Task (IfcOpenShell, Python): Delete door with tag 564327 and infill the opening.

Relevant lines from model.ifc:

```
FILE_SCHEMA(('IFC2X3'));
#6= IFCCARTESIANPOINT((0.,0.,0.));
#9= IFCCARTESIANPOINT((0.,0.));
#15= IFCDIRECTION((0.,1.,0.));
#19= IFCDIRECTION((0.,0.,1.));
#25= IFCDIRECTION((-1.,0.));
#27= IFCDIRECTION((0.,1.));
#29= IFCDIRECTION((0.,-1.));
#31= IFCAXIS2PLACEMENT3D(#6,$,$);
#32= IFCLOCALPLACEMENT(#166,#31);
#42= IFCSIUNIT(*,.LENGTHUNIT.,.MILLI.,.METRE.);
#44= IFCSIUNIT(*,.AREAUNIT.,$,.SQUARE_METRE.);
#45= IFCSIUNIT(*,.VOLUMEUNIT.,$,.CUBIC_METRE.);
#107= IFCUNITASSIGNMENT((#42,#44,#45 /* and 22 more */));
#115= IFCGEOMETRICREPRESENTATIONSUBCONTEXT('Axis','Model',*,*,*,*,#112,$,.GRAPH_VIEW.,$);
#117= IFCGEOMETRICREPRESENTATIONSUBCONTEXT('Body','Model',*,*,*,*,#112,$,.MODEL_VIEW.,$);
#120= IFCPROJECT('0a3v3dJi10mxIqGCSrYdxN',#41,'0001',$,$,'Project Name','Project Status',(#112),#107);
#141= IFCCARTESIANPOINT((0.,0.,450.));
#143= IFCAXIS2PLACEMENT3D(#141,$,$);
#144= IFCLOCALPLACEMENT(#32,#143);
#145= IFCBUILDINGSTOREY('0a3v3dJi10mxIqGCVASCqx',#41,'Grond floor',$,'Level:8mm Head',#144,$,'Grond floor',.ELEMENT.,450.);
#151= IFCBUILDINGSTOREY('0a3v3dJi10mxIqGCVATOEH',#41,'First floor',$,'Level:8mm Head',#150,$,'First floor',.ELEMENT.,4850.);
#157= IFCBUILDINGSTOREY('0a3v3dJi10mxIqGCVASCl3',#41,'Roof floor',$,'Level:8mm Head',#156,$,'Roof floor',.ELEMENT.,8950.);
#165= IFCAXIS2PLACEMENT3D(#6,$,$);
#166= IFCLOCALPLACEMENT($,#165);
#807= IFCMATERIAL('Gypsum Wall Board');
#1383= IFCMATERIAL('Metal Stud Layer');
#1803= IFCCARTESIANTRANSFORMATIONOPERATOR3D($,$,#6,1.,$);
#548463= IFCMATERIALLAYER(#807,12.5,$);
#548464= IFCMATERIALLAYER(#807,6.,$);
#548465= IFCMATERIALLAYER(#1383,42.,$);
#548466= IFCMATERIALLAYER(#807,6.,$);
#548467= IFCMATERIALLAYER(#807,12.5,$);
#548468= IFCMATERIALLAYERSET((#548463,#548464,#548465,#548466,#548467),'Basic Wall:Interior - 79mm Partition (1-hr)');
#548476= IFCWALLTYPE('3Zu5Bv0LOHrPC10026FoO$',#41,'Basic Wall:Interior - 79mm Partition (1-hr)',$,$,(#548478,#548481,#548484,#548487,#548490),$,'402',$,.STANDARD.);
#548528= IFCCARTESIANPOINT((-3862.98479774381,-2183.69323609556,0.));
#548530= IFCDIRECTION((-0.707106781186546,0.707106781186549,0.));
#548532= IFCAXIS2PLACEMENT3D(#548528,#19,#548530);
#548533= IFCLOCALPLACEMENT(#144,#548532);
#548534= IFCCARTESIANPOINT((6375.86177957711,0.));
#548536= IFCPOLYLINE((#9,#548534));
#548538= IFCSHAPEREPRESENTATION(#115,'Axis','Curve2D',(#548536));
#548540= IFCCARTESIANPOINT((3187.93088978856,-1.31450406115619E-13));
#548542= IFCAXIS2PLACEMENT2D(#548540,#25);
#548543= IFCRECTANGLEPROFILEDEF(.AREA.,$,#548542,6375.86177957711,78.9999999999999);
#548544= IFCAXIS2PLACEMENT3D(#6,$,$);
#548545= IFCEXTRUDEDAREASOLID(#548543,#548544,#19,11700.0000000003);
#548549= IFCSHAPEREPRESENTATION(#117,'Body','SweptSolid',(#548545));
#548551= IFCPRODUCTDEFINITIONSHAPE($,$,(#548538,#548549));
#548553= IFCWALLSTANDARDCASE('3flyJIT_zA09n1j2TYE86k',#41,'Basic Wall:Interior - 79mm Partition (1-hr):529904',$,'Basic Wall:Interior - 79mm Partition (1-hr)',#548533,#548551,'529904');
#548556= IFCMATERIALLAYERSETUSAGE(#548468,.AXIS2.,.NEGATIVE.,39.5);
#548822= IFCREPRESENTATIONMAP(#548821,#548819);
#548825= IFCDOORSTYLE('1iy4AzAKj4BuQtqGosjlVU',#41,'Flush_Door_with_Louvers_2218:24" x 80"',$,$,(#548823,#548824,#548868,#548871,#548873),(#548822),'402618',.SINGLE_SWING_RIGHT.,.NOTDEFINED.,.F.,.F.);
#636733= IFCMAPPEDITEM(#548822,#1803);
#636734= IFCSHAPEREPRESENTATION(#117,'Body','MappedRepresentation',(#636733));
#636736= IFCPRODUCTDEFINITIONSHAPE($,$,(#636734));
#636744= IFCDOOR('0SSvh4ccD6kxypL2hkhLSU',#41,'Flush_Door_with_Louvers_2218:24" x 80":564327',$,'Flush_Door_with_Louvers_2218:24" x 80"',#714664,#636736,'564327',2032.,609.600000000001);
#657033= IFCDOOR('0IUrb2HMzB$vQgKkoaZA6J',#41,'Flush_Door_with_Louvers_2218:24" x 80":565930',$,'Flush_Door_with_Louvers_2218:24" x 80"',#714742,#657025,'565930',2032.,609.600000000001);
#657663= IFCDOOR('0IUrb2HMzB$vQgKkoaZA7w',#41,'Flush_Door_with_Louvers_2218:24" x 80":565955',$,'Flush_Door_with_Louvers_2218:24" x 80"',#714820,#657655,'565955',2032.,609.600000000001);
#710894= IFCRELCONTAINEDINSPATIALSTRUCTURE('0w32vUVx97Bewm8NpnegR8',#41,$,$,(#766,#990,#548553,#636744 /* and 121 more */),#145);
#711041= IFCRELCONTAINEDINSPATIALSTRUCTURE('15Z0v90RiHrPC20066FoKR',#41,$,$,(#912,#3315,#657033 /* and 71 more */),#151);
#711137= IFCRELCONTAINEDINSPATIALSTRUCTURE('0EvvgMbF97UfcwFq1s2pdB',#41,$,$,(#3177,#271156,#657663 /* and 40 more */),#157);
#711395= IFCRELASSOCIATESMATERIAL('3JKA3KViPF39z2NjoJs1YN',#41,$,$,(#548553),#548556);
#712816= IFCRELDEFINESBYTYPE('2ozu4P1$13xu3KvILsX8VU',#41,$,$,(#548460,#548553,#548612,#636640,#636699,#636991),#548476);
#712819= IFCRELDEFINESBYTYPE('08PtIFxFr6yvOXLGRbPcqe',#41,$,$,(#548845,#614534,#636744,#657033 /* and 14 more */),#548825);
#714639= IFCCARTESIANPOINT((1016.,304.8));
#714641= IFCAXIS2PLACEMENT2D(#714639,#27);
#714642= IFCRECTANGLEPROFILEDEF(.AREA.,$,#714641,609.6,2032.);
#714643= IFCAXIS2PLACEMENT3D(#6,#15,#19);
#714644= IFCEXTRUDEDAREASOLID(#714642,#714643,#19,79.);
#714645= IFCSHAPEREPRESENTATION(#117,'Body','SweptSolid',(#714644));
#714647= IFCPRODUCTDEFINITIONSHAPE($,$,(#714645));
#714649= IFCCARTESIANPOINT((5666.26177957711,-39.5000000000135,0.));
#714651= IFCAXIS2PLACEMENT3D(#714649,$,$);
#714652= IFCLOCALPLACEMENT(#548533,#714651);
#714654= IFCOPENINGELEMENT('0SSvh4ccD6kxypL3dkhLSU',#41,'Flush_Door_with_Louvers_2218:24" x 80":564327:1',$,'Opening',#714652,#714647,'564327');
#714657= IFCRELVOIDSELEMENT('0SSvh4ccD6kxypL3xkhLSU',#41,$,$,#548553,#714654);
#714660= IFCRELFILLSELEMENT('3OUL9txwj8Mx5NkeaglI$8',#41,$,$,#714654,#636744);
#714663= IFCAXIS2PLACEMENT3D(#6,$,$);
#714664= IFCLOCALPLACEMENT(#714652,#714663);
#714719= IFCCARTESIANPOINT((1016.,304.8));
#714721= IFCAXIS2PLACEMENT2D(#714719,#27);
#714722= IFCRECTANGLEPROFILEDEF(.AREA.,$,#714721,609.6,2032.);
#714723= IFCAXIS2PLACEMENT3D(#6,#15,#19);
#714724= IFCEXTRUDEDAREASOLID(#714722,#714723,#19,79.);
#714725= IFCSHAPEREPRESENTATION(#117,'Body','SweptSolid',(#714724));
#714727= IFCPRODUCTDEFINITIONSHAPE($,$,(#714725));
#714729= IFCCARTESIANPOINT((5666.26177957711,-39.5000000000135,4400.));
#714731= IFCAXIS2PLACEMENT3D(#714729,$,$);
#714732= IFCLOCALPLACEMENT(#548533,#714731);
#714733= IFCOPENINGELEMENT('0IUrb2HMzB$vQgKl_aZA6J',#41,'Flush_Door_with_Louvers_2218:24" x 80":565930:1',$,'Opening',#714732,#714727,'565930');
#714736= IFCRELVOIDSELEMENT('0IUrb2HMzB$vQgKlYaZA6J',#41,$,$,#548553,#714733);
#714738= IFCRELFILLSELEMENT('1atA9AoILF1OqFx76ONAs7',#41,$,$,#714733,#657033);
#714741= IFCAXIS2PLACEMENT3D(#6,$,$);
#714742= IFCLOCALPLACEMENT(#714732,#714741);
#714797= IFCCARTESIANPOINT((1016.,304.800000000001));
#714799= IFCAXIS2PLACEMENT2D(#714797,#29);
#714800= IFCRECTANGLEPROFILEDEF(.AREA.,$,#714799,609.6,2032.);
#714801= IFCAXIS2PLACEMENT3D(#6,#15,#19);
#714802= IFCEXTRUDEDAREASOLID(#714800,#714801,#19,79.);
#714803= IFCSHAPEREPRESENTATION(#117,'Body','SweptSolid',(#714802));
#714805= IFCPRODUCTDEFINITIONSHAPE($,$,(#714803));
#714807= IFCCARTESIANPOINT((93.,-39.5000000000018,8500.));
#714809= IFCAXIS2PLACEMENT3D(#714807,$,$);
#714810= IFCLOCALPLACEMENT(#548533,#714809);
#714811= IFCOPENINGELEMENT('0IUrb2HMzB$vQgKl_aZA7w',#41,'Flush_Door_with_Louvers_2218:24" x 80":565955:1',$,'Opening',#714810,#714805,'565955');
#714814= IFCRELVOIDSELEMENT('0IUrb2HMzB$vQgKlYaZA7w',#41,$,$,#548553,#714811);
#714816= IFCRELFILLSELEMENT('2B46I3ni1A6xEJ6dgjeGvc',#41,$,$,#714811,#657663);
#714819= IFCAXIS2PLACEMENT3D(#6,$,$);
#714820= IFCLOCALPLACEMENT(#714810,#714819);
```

```python
import ifcopenshell
import ifcopenshell.api.feature
import ifcopenshell.api.root
import ifcopenshell.geom
import ifcopenshell.util.shape

model = ifcopenshell.open("model.ifc")
settings = ifcopenshell.geom.settings()


def volume(element):
    """Net volume in cubic metres, openings subtracted."""
    shape = ifcopenshell.geom.create_shape(settings, element)
    return ifcopenshell.util.shape.get_volume(shape.geometry)


door = model.by_id(636744)
opening = door.FillsVoids[0].RelatingOpeningElement
wall = opening.VoidsElements[0].RelatingBuildingElement
before = volume(wall)

ifcopenshell.api.root.remove_product(model, product=door)
ifcopenshell.api.feature.remove_feature(model, feature=opening)

after = volume(wall)

print(f"wall volume {before:.3f} -> {after:.3f} m3")

model.write("model-out.ifc")
```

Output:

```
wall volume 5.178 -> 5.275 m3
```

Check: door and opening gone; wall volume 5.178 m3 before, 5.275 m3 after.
